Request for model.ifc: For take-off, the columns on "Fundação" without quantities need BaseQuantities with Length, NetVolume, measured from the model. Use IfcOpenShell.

First a look at what the model holds.

```python
import ifcopenshell
import ifcopenshell.util.element
import ifcopenshell.util.unit

model = ifcopenshell.open("model.ifc")
print(model.schema)
for unit_type in ("LENGTHUNIT", "AREAUNIT", "VOLUMEUNIT"):
    print(unit_type, ifcopenshell.util.unit.calculate_unit_scale(model, unit_type))
storey = next(s for s in model.by_type("IfcBuildingStorey") if s.Name == "Fundação")
columns = [e for e in ifcopenshell.util.element.get_decomposition(storey) if e.is_a("IfcColumn")]
for e in sorted(columns, key=lambda e: e.id()):
    print(e.id(), e.is_a(), e.Name, list(ifcopenshell.util.element.get_psets(e, qtos_only=True)), sep=" | ")
```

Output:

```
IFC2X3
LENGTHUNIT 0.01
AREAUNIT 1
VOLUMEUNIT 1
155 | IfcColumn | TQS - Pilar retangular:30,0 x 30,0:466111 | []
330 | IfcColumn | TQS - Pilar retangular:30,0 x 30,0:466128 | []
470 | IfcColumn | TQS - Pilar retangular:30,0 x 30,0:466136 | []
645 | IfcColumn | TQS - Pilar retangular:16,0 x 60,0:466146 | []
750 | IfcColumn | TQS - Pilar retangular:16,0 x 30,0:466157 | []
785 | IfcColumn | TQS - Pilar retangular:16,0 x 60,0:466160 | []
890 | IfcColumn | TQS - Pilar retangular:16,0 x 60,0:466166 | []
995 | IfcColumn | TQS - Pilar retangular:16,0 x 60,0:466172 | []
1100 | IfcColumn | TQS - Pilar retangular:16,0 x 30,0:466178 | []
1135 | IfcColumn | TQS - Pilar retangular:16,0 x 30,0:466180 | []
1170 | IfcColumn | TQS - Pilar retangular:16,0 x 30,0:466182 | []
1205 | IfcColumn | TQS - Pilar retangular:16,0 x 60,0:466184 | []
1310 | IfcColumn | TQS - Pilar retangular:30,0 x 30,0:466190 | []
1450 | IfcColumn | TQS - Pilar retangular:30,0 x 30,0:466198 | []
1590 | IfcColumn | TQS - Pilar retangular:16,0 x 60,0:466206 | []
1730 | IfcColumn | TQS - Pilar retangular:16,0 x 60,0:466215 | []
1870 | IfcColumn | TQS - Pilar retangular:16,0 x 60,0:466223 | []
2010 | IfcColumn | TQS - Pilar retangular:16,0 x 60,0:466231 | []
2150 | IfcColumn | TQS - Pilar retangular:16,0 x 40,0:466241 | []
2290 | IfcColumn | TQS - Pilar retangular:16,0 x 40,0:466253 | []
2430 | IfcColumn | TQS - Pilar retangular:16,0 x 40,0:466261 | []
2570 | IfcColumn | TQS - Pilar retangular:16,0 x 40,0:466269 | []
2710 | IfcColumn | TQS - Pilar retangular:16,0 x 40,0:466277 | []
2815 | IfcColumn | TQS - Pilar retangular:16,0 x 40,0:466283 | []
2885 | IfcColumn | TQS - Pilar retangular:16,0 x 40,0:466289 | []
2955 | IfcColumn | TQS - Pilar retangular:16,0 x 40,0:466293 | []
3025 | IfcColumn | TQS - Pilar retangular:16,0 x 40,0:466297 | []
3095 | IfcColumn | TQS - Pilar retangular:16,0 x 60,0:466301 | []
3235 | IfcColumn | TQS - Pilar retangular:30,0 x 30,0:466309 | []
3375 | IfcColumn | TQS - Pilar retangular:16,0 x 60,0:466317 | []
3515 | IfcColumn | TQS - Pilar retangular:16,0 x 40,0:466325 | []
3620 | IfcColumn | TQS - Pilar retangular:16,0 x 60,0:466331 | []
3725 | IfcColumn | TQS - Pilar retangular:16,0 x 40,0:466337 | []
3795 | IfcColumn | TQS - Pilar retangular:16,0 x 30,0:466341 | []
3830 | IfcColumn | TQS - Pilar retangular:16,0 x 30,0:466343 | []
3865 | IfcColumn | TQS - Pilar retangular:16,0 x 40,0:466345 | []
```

```python
import ifcopenshell
import ifcopenshell.api.pset
import ifcopenshell.geom
import ifcopenshell.util.element
import ifcopenshell.util.shape
import ifcopenshell.util.unit

model = ifcopenshell.open("model.ifc")
unit_scale = ifcopenshell.util.unit.calculate_unit_scale(model)
volume_scale = ifcopenshell.util.unit.calculate_unit_scale(model, "VOLUMEUNIT")
settings = ifcopenshell.geom.settings()

storey = next(s for s in model.by_type("IfcBuildingStorey") if s.Name == "Fundação")
columns = [e for e in ifcopenshell.util.element.get_decomposition(storey) if e.is_a("IfcColumn")]

for e in sorted(columns, key=lambda e: e.id()):
    if ifcopenshell.util.element.get_psets(e, qtos_only=True, should_inherit=False):
        continue
    # Geometry comes back in metres, in the element's own axes.
    shape = ifcopenshell.geom.create_shape(settings, e)
    values = {
        "Length": ifcopenshell.util.shape.get_z(shape.geometry) / unit_scale,
        "NetVolume": ifcopenshell.util.shape.get_volume(shape.geometry) / volume_scale,
    }
    qto = ifcopenshell.api.pset.add_qto(model, product=e, name="BaseQuantities")
    ifcopenshell.api.pset.edit_qto(model, qto=qto, properties=values)
    print(e.id(), {k: round(v, 3) for k, v in values.items()})

model.write("model_rev.ifc")
```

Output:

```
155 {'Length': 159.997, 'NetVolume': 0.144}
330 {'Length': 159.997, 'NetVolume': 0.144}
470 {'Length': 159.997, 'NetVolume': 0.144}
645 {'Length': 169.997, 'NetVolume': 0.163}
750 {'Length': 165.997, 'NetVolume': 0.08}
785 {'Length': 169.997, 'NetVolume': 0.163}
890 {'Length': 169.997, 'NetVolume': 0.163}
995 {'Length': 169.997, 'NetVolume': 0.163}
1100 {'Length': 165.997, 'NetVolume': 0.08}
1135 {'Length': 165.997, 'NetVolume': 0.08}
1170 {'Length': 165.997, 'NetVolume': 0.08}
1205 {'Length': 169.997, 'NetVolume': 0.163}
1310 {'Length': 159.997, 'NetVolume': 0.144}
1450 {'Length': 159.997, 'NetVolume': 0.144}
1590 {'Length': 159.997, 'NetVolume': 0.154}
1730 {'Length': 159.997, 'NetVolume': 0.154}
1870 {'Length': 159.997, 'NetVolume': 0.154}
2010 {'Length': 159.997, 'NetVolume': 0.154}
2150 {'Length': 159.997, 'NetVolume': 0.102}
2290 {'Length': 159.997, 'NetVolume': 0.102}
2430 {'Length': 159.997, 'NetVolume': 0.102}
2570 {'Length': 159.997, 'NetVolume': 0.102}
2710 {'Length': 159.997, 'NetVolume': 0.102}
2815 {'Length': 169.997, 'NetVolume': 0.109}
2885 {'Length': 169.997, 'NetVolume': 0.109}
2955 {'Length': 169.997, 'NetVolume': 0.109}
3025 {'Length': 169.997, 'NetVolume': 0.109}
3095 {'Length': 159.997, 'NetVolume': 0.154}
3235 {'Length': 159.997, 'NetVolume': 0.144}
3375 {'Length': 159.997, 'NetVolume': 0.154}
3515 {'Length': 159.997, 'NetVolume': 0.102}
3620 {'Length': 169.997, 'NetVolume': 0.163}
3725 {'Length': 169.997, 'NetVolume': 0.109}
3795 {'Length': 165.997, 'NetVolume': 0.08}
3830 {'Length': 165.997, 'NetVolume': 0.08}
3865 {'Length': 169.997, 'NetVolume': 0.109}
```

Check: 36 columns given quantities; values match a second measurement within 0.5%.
